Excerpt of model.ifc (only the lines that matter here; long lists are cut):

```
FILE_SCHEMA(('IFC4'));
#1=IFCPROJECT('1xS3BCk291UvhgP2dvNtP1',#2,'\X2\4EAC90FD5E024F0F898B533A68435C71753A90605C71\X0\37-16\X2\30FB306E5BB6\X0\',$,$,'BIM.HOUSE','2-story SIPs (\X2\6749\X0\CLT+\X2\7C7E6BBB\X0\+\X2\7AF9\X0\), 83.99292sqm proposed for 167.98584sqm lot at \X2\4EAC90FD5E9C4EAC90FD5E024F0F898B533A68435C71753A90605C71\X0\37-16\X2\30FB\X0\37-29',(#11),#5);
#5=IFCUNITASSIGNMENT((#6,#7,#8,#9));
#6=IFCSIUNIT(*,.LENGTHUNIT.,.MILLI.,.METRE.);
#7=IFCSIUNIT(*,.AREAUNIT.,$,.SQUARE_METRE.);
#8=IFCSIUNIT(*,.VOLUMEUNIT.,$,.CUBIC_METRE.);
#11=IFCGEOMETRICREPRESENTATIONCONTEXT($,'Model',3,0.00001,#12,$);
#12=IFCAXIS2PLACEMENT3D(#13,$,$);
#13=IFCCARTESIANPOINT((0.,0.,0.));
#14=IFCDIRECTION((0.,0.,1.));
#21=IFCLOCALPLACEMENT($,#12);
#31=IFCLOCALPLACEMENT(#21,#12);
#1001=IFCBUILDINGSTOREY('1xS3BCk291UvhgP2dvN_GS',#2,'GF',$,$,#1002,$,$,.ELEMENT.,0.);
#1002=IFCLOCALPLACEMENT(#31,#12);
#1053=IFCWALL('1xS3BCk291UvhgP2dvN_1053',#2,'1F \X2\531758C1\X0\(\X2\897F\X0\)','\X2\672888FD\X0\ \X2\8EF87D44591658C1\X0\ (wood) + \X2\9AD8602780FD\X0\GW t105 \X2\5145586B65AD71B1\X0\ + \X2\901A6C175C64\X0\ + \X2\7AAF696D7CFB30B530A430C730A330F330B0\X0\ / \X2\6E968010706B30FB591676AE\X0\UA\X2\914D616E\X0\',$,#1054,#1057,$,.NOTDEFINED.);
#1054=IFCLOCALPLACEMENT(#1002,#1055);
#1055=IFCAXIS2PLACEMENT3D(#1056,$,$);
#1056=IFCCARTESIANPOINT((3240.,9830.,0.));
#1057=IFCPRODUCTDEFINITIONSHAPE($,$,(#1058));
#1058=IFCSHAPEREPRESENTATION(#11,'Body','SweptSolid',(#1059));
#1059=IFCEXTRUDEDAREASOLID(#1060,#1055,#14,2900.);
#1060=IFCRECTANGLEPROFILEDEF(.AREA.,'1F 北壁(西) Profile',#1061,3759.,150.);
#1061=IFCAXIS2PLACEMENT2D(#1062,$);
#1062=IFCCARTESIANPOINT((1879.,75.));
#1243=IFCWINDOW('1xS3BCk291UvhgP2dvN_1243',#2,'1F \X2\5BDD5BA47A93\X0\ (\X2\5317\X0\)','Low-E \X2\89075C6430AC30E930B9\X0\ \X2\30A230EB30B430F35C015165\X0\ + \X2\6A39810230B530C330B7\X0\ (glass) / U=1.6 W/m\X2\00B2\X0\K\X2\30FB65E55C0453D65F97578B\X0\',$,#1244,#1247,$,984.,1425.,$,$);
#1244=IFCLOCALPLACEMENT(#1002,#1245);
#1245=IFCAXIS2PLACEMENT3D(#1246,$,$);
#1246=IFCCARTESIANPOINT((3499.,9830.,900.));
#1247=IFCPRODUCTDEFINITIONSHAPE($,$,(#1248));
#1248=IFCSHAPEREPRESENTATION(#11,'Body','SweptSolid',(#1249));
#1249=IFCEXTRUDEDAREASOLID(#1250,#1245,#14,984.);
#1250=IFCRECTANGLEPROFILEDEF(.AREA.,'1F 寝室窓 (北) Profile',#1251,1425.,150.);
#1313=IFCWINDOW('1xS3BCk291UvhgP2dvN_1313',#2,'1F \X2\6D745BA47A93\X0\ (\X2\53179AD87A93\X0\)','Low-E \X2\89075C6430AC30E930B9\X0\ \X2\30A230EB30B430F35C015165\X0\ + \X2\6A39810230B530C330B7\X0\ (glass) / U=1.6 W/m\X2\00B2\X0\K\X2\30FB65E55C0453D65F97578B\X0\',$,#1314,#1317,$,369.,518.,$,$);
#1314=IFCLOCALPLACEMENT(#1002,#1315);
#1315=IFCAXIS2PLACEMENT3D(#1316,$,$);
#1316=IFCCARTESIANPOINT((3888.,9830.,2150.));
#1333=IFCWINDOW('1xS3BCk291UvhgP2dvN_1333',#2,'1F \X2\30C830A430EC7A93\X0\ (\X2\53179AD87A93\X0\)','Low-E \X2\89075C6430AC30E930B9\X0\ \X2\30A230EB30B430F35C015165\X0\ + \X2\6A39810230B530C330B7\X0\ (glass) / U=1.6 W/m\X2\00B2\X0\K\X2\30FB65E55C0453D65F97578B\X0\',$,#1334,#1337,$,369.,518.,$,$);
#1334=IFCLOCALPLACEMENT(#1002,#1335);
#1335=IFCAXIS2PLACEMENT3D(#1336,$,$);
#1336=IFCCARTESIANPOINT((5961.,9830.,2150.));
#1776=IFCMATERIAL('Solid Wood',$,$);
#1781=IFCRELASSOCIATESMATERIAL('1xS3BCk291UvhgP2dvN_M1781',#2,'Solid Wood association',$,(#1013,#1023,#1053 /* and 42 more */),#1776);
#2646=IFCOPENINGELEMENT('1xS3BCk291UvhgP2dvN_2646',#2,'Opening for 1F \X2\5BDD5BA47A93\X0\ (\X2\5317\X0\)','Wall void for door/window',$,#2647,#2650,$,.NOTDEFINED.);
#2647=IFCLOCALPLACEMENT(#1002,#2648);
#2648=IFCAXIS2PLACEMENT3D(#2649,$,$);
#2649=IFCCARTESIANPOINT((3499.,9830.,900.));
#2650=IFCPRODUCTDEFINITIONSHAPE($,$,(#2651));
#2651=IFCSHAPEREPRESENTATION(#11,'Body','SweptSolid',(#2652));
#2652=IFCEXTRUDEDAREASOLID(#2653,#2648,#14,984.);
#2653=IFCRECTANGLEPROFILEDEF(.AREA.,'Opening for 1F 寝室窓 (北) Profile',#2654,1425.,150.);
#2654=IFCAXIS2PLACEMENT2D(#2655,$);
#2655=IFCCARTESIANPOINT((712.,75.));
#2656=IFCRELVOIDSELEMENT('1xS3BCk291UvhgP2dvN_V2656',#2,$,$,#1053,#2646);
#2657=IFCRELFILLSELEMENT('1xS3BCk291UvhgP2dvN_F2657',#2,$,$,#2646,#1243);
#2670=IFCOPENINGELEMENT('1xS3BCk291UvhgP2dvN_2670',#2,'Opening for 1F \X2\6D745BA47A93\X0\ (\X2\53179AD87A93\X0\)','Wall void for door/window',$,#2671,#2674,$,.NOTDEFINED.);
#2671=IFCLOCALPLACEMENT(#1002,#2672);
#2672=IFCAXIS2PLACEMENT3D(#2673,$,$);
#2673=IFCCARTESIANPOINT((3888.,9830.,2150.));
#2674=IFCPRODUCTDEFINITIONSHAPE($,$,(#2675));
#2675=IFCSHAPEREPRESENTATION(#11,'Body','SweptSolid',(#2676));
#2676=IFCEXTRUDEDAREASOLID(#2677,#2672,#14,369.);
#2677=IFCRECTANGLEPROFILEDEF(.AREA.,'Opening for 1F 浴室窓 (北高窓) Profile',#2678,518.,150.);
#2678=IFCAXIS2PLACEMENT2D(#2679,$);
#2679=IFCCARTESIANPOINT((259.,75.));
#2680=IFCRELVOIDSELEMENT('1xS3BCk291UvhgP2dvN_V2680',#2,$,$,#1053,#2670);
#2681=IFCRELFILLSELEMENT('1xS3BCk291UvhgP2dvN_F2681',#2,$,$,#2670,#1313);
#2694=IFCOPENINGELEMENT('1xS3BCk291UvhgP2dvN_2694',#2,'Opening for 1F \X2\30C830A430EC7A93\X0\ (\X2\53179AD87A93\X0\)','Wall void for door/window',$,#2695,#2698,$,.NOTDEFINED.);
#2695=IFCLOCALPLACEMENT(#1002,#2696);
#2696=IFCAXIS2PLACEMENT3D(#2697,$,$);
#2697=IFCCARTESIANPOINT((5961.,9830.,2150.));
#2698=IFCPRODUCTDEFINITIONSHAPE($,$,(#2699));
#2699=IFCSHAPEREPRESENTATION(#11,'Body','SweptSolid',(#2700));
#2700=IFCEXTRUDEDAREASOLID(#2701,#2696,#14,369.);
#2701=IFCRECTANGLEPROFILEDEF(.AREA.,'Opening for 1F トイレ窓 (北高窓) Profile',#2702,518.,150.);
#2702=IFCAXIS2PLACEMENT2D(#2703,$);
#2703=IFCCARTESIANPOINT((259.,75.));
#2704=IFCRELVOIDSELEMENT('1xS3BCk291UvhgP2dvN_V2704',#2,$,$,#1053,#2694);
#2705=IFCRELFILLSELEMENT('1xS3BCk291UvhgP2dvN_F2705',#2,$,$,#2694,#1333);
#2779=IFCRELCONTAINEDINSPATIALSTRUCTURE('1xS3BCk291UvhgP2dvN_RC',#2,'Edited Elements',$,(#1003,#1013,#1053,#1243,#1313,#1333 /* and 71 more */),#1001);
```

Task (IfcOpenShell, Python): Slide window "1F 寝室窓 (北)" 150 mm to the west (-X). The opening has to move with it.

```python
import ifcopenshell
import ifcopenshell.api.geometry
import ifcopenshell.util.placement
import ifcopenshell.util.unit

model = ifcopenshell.open("model.ifc")
unit_scale = ifcopenshell.util.unit.calculate_unit_scale(model)

window = model.by_guid("1xS3BCk291UvhgP2dvN_1243")
opening = window.FillsVoids[0].RelatingOpeningElement
wall = opening.VoidsElements[0].RelatingBuildingElement

wall_matrix = ifcopenshell.util.placement.get_local_placement(wall.ObjectPlacement)
shift = wall_matrix[:3, 0] * -0.15 / unit_scale
before = ifcopenshell.util.placement.get_local_placement(window.ObjectPlacement)[:3, 3].copy()

# The window is not placed relative to its opening, so move both.
for product in (opening, window):
    matrix = ifcopenshell.util.placement.get_local_placement(product.ObjectPlacement)
    matrix[:3, 3] += shift
    ifcopenshell.api.geometry.edit_object_placement(model, product=product, matrix=matrix, is_si=False)

after = ifcopenshell.util.placement.get_local_placement(window.ObjectPlacement)[:3, 3]
print("window moved by", (after - before).round(3) + 0.0)

model.write("model_updated.ifc")
```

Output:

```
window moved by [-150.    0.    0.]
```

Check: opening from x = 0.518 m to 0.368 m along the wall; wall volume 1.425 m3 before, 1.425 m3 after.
